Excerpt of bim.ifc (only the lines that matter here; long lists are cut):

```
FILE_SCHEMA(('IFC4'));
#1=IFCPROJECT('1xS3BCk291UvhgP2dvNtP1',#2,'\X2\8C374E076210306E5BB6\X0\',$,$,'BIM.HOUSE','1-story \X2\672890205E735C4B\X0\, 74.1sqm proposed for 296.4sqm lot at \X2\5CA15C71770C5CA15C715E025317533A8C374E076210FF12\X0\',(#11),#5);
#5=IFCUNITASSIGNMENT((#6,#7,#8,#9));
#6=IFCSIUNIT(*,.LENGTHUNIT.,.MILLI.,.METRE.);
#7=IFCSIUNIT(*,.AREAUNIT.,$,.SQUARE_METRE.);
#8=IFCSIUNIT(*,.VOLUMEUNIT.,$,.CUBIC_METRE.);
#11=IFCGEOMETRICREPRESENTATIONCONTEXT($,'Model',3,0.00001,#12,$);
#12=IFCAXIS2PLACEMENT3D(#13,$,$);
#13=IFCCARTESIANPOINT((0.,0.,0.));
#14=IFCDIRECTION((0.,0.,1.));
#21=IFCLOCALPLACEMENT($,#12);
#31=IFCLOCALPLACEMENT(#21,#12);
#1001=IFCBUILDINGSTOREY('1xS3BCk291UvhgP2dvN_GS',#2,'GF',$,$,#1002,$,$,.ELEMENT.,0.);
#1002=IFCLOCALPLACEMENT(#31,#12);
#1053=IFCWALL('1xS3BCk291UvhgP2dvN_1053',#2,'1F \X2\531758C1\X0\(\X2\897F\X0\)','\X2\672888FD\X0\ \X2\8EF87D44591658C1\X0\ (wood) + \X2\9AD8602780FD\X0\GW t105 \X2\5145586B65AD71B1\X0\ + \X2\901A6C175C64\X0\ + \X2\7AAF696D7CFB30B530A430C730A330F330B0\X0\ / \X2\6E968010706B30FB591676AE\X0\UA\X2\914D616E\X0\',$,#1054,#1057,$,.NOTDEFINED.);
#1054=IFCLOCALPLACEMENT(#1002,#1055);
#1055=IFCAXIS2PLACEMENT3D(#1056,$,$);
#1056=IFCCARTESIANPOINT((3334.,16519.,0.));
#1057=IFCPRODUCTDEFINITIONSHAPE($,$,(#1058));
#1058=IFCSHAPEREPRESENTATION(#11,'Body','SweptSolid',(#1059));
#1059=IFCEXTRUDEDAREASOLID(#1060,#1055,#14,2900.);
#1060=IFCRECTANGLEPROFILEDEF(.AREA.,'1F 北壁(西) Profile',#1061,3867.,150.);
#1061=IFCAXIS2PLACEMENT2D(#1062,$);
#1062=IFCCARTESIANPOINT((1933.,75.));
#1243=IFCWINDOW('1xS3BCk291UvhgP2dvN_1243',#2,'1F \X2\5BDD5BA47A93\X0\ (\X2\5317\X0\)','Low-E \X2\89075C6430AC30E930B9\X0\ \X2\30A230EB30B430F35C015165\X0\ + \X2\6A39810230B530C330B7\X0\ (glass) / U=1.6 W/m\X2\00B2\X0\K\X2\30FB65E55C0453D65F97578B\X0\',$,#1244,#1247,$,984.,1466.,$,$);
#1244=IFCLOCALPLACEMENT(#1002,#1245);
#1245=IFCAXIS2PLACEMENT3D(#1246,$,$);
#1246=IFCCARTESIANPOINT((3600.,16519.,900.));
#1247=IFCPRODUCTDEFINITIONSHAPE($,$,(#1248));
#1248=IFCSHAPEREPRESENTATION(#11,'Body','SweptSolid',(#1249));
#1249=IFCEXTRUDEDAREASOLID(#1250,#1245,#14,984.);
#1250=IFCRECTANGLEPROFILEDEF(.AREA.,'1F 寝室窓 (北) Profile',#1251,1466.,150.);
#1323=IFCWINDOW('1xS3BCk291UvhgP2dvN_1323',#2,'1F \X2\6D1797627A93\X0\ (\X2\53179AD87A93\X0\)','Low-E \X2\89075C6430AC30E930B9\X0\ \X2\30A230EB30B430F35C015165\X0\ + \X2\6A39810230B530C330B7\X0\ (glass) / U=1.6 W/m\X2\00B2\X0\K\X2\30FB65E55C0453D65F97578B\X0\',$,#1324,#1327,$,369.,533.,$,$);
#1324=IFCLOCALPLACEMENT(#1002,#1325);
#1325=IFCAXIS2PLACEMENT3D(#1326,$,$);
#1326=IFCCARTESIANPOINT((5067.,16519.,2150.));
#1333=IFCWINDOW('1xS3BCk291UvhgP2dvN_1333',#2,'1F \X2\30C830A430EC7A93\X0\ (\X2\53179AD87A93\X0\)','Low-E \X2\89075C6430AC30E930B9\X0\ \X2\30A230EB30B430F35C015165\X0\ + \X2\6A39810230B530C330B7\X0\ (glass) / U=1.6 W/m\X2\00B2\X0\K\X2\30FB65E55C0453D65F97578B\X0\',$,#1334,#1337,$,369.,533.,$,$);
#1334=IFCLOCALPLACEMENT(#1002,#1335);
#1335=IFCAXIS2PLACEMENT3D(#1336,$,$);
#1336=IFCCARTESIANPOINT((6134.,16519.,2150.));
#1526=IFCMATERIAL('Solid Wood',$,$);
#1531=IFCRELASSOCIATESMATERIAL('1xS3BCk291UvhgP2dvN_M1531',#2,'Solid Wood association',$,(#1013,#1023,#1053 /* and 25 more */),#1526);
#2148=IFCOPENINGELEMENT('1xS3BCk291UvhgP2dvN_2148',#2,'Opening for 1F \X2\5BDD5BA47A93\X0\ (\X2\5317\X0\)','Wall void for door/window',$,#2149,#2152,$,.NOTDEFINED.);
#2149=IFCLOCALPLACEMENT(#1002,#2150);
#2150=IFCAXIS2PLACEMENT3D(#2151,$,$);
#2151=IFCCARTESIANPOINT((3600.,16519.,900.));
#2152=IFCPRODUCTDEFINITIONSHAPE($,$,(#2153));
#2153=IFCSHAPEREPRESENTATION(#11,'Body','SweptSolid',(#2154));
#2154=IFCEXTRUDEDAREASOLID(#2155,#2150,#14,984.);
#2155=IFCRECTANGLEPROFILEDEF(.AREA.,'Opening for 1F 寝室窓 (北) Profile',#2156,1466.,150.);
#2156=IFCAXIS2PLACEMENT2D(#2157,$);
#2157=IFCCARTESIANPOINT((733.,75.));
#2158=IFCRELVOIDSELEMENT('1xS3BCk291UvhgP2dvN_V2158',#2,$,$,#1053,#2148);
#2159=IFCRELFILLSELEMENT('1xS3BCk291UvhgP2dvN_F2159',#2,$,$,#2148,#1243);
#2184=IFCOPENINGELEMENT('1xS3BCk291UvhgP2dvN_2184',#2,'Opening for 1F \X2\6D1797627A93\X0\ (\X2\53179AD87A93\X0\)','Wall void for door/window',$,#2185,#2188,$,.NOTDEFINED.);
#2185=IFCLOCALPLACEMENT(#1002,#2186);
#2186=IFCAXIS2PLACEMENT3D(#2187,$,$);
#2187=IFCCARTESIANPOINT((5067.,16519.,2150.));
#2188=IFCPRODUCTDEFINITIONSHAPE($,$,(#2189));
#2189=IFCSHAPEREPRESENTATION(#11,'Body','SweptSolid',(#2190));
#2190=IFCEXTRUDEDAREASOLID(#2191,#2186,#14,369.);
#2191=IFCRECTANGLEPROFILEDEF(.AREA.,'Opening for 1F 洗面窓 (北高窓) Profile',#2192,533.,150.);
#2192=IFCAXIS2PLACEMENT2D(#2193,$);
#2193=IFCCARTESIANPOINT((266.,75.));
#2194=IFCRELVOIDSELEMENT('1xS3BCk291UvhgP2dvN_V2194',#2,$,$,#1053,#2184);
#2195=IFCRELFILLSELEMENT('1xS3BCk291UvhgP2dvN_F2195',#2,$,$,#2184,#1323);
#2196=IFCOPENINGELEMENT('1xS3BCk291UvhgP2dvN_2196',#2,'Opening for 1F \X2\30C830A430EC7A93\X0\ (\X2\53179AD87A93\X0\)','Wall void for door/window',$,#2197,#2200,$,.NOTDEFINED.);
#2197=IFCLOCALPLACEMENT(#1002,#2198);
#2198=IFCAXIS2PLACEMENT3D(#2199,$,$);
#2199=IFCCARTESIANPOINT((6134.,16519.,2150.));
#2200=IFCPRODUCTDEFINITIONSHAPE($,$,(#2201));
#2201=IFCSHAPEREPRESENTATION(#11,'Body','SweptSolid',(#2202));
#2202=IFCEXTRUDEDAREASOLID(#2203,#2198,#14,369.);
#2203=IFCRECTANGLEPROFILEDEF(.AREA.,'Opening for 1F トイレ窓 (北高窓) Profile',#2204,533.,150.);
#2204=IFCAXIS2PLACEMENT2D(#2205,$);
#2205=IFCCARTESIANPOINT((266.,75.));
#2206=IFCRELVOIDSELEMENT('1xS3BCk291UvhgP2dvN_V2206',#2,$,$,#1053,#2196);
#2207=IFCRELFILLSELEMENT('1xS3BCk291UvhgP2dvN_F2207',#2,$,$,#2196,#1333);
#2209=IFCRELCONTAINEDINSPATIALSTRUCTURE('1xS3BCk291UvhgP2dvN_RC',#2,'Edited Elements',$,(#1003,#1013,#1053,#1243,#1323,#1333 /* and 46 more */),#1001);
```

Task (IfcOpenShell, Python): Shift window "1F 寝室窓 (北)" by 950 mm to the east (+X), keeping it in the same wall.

```python
import ifcopenshell
import ifcopenshell.api.geometry
import ifcopenshell.util.placement

model = ifcopenshell.open("bim.ifc")

window = model.by_guid("1xS3BCk291UvhgP2dvN_1243")
opening = window.FillsVoids[0].RelatingOpeningElement
wall = opening.VoidsElements[0].RelatingBuildingElement

wall_matrix = ifcopenshell.util.placement.get_local_placement(wall.ObjectPlacement)
shift = wall_matrix[:3, 0] * 950.0
before = ifcopenshell.util.placement.get_local_placement(window.ObjectPlacement)[:3, 3].copy()

# The window is not placed relative to its opening, so move both.
for product in (opening, window):
    matrix = ifcopenshell.util.placement.get_local_placement(product.ObjectPlacement)
    matrix[:3, 3] += shift
    ifcopenshell.api.geometry.edit_object_placement(model, product=product, matrix=matrix, is_si=False)

after = ifcopenshell.util.placement.get_local_placement(window.ObjectPlacement)[:3, 3]
print("window moved by", (after - before).round(3) + 0.0)

model.write("bim_v2.ifc")
```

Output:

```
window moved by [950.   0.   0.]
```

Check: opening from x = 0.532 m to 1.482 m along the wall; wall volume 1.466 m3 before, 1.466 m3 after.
